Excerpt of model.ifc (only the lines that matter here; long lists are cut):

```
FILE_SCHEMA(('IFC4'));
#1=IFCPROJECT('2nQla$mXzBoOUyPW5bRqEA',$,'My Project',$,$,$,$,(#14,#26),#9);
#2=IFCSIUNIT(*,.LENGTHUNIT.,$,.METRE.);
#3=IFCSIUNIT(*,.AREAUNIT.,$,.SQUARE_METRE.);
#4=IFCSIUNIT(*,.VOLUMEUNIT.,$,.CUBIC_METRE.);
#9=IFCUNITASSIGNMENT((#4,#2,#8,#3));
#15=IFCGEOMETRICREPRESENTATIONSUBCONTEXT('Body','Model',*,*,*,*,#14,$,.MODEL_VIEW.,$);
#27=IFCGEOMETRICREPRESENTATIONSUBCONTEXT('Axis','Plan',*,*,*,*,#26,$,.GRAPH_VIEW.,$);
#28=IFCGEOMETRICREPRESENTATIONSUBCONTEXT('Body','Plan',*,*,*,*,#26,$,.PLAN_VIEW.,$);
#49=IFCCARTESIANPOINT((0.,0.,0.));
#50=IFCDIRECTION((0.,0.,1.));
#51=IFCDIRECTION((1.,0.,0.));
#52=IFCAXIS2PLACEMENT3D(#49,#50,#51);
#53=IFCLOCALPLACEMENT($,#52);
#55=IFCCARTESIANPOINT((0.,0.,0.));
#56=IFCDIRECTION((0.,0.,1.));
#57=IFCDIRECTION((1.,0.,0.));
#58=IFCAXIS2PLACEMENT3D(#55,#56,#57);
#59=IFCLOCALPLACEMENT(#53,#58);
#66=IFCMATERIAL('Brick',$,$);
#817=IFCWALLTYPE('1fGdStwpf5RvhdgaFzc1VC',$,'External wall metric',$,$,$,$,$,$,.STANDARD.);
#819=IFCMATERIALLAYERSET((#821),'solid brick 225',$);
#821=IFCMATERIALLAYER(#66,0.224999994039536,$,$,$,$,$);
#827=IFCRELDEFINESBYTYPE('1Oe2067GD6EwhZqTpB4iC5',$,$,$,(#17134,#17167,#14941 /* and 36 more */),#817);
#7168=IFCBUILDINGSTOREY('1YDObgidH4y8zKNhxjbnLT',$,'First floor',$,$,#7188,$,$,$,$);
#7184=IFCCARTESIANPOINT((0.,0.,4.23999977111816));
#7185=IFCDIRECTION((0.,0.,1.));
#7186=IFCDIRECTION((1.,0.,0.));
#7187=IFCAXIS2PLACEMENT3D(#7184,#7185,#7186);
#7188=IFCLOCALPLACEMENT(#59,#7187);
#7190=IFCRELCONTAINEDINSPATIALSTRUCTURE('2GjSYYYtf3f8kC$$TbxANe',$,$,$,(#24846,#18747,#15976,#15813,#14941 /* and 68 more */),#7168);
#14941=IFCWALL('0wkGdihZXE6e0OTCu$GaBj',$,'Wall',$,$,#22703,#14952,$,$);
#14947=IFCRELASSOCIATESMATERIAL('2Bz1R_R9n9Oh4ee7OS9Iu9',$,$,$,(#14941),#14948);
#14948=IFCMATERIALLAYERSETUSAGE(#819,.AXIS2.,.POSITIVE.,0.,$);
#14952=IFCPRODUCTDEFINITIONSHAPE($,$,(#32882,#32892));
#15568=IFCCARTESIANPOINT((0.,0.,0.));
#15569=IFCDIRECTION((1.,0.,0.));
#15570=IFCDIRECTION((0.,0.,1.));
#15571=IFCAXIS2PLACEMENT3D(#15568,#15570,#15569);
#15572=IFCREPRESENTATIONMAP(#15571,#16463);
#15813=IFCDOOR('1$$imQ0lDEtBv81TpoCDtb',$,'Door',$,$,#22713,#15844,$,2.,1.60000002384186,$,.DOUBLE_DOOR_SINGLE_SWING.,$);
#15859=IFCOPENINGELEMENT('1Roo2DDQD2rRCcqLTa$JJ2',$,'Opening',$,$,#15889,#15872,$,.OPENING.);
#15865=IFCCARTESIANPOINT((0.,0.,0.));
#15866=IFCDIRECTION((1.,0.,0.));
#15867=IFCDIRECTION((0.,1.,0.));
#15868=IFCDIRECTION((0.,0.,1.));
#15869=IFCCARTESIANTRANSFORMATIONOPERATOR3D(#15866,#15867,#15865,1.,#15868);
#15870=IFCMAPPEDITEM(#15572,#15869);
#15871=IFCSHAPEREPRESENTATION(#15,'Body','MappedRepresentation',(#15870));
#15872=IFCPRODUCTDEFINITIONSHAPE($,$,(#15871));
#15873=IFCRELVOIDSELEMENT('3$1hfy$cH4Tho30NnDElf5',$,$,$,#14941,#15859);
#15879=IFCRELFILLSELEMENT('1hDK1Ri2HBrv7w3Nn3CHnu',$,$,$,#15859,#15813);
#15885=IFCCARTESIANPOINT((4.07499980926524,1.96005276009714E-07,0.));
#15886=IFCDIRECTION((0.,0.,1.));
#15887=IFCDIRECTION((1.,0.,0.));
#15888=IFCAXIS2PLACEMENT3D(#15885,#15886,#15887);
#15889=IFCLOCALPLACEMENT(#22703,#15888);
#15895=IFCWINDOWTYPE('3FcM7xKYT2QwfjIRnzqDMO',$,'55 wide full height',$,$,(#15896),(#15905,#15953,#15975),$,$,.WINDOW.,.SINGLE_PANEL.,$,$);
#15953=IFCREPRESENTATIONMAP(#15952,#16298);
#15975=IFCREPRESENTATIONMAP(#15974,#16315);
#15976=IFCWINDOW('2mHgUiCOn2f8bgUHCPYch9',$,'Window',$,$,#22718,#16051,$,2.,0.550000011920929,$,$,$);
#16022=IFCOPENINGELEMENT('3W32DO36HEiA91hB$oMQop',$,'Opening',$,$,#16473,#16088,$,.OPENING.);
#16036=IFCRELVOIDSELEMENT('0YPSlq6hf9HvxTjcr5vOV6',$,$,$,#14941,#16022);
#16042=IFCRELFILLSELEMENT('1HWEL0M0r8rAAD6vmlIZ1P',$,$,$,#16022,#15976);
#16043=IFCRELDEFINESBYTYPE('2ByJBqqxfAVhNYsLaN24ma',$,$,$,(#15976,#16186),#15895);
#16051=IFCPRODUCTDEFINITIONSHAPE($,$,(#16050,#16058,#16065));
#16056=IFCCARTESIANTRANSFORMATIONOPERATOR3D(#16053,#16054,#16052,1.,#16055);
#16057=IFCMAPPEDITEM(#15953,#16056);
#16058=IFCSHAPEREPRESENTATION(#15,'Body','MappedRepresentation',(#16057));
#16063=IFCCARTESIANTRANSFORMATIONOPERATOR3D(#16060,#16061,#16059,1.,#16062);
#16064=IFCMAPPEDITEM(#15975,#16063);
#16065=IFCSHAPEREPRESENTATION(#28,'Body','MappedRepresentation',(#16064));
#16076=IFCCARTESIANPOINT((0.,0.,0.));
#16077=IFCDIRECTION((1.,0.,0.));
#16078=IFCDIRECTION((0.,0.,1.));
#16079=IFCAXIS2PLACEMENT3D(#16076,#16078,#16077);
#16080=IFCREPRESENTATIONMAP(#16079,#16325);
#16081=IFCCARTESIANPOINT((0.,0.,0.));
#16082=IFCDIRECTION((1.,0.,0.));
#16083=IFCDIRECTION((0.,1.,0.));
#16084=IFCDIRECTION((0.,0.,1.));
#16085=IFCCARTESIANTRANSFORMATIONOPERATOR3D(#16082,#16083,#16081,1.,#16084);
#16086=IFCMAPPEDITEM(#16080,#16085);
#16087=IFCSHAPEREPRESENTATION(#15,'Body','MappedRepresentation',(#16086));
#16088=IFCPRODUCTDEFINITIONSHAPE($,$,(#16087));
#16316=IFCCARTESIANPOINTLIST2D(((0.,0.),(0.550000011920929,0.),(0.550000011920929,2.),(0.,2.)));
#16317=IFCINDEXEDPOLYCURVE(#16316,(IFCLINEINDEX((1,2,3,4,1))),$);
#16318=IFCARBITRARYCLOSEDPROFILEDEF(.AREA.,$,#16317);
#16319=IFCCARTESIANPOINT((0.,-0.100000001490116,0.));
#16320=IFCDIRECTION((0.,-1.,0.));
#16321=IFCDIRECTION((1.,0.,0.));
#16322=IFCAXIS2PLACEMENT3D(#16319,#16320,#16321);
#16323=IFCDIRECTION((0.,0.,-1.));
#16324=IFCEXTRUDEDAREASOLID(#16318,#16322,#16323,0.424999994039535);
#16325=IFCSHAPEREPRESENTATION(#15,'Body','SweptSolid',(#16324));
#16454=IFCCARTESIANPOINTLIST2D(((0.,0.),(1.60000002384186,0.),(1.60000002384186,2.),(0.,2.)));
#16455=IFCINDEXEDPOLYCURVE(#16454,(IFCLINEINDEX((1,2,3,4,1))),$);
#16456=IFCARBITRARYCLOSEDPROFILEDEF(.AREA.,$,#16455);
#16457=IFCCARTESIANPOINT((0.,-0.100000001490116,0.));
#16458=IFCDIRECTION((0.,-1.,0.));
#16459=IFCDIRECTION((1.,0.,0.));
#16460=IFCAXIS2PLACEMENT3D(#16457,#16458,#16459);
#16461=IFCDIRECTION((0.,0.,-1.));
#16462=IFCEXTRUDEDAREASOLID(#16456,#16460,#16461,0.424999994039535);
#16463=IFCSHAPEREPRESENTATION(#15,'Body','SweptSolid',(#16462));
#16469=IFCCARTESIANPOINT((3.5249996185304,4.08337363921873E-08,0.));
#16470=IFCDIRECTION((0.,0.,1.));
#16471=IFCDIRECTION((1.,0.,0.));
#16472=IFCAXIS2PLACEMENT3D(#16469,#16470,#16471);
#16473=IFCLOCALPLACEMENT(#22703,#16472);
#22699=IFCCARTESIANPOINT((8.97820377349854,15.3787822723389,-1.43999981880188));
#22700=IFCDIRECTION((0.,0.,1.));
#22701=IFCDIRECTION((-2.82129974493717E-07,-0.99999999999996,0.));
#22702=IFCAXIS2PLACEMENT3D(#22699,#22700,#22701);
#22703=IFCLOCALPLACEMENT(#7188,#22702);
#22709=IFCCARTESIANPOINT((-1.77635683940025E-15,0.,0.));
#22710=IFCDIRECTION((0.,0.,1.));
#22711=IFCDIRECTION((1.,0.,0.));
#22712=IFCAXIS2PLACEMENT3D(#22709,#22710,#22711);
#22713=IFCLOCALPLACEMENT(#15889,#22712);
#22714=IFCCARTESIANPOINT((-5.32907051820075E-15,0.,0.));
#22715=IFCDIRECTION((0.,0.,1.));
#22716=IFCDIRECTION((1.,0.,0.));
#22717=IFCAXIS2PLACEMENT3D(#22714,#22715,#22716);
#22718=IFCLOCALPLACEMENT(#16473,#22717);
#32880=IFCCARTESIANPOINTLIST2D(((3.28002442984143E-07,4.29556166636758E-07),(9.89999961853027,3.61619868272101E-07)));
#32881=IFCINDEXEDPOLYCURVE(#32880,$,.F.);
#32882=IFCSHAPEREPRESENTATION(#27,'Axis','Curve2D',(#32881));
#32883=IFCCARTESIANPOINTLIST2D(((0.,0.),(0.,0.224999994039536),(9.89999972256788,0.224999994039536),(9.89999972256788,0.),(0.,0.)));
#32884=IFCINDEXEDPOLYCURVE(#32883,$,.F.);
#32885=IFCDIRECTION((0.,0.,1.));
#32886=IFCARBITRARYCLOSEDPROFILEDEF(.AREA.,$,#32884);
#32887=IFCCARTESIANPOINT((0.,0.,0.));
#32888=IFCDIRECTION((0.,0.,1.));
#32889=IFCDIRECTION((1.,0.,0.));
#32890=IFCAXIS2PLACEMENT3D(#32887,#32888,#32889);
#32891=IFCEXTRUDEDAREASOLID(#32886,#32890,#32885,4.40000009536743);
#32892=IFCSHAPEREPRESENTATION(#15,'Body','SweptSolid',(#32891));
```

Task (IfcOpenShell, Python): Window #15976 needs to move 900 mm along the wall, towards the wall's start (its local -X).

```python
import ifcopenshell
import ifcopenshell.api.geometry
import ifcopenshell.util.placement

model = ifcopenshell.open("model.ifc")

window = model.by_id(15976)
opening = window.FillsVoids[0].RelatingOpeningElement
wall = opening.VoidsElements[0].RelatingBuildingElement

wall_matrix = ifcopenshell.util.placement.get_local_placement(wall.ObjectPlacement)
shift = wall_matrix[:3, 0] * -0.9
before = ifcopenshell.util.placement.get_local_placement(window.ObjectPlacement)[:3, 3].copy()

# The window is placed relative to its opening, so it follows when the opening moves.
matrix = ifcopenshell.util.placement.get_local_placement(opening.ObjectPlacement)
matrix[:3, 3] += shift
ifcopenshell.api.geometry.edit_object_placement(
    model, product=opening, matrix=matrix, is_si=False, should_transform_children=True
)

after = ifcopenshell.util.placement.get_local_placement(window.ObjectPlacement)[:3, 3]
print("window moved by", (after - before).round(3) + 0.0)

model.write("model_edited.ifc")
```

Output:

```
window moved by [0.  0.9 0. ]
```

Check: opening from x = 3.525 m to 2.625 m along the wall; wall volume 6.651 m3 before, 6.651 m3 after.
